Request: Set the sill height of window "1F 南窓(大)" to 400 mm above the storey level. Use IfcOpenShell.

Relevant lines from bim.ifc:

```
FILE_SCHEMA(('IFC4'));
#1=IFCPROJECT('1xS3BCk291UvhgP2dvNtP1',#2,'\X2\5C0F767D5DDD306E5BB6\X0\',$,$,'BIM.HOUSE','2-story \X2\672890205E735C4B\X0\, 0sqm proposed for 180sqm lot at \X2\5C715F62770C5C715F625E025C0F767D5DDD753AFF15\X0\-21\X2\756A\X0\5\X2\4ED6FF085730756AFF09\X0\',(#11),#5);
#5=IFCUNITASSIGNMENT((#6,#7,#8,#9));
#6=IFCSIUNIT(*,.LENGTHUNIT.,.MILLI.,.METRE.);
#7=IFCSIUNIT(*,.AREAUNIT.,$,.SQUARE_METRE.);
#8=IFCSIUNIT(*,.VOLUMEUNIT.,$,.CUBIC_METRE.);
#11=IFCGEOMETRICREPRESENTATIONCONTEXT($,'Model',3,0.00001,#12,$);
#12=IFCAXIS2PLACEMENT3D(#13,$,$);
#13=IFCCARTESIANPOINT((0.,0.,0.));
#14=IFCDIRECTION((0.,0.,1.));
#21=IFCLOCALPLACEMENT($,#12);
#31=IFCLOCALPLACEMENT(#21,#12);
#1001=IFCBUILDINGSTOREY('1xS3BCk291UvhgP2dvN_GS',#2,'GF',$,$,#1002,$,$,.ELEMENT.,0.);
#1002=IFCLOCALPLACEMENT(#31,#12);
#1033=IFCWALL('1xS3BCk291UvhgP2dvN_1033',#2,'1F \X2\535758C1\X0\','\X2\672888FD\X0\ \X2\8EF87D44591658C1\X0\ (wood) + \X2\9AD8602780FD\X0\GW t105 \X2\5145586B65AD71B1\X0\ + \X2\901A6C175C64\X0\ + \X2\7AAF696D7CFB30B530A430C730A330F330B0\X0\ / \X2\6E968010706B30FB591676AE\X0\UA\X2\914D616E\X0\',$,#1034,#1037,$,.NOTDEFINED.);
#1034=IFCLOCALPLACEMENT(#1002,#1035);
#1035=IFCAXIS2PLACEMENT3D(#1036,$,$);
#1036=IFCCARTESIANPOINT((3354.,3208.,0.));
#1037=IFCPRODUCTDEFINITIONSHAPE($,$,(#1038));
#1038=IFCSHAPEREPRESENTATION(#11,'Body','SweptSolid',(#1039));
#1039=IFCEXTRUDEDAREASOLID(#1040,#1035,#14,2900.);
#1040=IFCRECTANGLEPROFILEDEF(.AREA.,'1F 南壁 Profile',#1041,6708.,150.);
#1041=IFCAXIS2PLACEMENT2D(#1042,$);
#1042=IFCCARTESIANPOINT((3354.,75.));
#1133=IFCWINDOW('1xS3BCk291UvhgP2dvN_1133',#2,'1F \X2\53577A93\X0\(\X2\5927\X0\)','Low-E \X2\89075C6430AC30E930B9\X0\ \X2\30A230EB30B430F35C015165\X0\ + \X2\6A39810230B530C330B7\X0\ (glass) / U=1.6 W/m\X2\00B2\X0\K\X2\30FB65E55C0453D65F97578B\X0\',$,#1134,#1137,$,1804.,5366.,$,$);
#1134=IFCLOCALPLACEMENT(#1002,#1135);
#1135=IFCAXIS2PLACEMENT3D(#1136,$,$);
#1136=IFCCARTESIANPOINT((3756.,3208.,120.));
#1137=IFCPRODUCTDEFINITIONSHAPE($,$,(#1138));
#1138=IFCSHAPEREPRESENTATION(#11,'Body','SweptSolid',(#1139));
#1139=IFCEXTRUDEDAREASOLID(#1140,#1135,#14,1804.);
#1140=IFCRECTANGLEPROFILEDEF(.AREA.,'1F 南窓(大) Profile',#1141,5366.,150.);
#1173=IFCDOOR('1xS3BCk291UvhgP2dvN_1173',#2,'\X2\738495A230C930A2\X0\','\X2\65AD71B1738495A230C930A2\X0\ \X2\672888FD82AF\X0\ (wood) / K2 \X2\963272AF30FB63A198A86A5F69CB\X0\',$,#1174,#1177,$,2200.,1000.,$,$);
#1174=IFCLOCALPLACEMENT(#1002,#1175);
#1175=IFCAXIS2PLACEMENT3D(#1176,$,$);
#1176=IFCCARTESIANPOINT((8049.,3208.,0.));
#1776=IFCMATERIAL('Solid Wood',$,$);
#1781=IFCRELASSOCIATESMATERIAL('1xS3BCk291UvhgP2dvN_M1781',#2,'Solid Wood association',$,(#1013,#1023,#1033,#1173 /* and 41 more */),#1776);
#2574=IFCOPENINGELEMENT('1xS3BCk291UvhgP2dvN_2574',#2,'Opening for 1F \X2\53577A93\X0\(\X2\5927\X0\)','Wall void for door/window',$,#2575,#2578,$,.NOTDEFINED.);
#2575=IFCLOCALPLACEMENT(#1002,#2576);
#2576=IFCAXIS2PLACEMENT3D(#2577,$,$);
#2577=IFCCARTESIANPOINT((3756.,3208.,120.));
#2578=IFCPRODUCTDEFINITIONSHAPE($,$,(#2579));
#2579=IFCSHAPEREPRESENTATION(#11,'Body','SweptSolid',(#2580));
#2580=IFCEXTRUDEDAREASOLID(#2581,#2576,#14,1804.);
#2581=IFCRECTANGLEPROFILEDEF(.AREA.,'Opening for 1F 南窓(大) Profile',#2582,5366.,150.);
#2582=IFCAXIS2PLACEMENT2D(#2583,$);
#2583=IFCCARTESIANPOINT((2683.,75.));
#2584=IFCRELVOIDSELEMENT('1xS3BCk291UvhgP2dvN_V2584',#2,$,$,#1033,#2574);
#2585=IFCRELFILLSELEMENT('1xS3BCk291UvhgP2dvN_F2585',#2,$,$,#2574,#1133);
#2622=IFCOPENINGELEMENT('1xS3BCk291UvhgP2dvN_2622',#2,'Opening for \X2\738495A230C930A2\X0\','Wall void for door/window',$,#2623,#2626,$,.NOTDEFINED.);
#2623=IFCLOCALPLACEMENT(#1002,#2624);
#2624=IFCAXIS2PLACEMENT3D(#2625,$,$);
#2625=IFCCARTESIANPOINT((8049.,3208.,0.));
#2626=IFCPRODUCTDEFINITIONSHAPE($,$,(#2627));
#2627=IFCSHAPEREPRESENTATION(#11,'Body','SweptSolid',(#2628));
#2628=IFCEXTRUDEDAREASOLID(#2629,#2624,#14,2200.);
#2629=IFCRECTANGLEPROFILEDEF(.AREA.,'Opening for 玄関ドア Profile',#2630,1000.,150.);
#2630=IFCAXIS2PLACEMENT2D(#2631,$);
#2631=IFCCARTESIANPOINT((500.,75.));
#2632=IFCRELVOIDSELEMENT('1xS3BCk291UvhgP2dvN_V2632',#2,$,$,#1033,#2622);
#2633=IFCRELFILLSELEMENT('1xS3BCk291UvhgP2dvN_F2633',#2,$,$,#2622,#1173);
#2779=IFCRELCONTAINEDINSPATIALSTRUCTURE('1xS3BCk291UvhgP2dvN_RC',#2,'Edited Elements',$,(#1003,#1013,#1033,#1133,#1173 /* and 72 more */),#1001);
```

```python
import numpy as np
import ifcopenshell
import ifcopenshell.api.geometry
import ifcopenshell.geom
import ifcopenshell.util.element
import ifcopenshell.util.placement
import ifcopenshell.util.shape
import ifcopenshell.util.unit

model = ifcopenshell.open("bim.ifc")
unit_scale = ifcopenshell.util.unit.calculate_unit_scale(model)

window = model.by_guid("1xS3BCk291UvhgP2dvN_1133")
opening = window.FillsVoids[0].RelatingOpeningElement
storey = ifcopenshell.util.element.get_container(window, ifc_class="IfcBuildingStorey")
level = ifcopenshell.util.placement.get_local_placement(storey.ObjectPlacement)[2, 3]

# The opening's origin need not be at the sill, so measure its lowest point.
shape = ifcopenshell.geom.create_shape(ifcopenshell.geom.settings(), opening)
bottom = ifcopenshell.util.shape.get_shape_bottom_elevation(shape, shape.geometry) / unit_scale
dz = level + 0.4 / unit_scale - bottom

shift = np.array([0.0, 0.0, dz])
# The window is not placed relative to its opening, so move both.
for product in (opening, window):
    matrix = ifcopenshell.util.placement.get_local_placement(product.ObjectPlacement)
    matrix[:3, 3] += shift
    ifcopenshell.api.geometry.edit_object_placement(model, product=product, matrix=matrix, is_si=False)

print(f"moved by {dz * unit_scale:+.3f} m")

model.write("bim_edited.ifc")
```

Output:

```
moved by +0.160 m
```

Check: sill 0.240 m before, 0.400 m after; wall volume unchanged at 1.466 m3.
